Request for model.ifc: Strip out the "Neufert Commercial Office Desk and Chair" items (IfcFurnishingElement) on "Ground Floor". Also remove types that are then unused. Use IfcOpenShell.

First a look at what the model holds.

```python
import ifcopenshell
import ifcopenshell.util.element

model = ifcopenshell.open("model.ifc")
print(model.schema)
storey = next(s for s in model.by_type("IfcBuildingStorey") if s.Name == "Ground Floor")
furniture = [e for e in ifcopenshell.util.element.get_decomposition(storey) if e.is_a("IfcFurnishingElement")]
seen = {}
for e in furniture:
    element_type = ifcopenshell.util.element.get_type(e)
    name = element_type.Name if element_type not in (None, e) else None
    seen[name] = seen.get(name, 0) + 1
for name, count in sorted(seen.items(), key=str):
    print(count, "x", name)
```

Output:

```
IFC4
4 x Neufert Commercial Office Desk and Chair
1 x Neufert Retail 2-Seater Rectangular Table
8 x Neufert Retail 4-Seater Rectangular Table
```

```python
import ifcopenshell
import ifcopenshell.api.root
import ifcopenshell.util.element

model = ifcopenshell.open("model.ifc")

storey = next(s for s in model.by_type("IfcBuildingStorey") if s.Name == "Ground Floor")
furniture = [e for e in ifcopenshell.util.element.get_decomposition(storey) if e.is_a("IfcFurnishingElement")]
targets = [e for e in furniture if (t := ifcopenshell.util.element.get_type(e)) not in (None, e) and t.Name == "Neufert Commercial Office Desk and Chair"]
types = {ifcopenshell.util.element.get_type(e) for e in targets} - {None, *targets}

for e in targets:
    ifcopenshell.api.root.remove_product(model, product=e)
print(len(targets), "removed")

unused = [t for t in types if not ifcopenshell.util.element.get_types(t)]
for t in unused:
    ifcopenshell.api.root.remove_product(model, product=t)
print(len(unused), "unused types removed")

model.write("model_updated.ifc")
```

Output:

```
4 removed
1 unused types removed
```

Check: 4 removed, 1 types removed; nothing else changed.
